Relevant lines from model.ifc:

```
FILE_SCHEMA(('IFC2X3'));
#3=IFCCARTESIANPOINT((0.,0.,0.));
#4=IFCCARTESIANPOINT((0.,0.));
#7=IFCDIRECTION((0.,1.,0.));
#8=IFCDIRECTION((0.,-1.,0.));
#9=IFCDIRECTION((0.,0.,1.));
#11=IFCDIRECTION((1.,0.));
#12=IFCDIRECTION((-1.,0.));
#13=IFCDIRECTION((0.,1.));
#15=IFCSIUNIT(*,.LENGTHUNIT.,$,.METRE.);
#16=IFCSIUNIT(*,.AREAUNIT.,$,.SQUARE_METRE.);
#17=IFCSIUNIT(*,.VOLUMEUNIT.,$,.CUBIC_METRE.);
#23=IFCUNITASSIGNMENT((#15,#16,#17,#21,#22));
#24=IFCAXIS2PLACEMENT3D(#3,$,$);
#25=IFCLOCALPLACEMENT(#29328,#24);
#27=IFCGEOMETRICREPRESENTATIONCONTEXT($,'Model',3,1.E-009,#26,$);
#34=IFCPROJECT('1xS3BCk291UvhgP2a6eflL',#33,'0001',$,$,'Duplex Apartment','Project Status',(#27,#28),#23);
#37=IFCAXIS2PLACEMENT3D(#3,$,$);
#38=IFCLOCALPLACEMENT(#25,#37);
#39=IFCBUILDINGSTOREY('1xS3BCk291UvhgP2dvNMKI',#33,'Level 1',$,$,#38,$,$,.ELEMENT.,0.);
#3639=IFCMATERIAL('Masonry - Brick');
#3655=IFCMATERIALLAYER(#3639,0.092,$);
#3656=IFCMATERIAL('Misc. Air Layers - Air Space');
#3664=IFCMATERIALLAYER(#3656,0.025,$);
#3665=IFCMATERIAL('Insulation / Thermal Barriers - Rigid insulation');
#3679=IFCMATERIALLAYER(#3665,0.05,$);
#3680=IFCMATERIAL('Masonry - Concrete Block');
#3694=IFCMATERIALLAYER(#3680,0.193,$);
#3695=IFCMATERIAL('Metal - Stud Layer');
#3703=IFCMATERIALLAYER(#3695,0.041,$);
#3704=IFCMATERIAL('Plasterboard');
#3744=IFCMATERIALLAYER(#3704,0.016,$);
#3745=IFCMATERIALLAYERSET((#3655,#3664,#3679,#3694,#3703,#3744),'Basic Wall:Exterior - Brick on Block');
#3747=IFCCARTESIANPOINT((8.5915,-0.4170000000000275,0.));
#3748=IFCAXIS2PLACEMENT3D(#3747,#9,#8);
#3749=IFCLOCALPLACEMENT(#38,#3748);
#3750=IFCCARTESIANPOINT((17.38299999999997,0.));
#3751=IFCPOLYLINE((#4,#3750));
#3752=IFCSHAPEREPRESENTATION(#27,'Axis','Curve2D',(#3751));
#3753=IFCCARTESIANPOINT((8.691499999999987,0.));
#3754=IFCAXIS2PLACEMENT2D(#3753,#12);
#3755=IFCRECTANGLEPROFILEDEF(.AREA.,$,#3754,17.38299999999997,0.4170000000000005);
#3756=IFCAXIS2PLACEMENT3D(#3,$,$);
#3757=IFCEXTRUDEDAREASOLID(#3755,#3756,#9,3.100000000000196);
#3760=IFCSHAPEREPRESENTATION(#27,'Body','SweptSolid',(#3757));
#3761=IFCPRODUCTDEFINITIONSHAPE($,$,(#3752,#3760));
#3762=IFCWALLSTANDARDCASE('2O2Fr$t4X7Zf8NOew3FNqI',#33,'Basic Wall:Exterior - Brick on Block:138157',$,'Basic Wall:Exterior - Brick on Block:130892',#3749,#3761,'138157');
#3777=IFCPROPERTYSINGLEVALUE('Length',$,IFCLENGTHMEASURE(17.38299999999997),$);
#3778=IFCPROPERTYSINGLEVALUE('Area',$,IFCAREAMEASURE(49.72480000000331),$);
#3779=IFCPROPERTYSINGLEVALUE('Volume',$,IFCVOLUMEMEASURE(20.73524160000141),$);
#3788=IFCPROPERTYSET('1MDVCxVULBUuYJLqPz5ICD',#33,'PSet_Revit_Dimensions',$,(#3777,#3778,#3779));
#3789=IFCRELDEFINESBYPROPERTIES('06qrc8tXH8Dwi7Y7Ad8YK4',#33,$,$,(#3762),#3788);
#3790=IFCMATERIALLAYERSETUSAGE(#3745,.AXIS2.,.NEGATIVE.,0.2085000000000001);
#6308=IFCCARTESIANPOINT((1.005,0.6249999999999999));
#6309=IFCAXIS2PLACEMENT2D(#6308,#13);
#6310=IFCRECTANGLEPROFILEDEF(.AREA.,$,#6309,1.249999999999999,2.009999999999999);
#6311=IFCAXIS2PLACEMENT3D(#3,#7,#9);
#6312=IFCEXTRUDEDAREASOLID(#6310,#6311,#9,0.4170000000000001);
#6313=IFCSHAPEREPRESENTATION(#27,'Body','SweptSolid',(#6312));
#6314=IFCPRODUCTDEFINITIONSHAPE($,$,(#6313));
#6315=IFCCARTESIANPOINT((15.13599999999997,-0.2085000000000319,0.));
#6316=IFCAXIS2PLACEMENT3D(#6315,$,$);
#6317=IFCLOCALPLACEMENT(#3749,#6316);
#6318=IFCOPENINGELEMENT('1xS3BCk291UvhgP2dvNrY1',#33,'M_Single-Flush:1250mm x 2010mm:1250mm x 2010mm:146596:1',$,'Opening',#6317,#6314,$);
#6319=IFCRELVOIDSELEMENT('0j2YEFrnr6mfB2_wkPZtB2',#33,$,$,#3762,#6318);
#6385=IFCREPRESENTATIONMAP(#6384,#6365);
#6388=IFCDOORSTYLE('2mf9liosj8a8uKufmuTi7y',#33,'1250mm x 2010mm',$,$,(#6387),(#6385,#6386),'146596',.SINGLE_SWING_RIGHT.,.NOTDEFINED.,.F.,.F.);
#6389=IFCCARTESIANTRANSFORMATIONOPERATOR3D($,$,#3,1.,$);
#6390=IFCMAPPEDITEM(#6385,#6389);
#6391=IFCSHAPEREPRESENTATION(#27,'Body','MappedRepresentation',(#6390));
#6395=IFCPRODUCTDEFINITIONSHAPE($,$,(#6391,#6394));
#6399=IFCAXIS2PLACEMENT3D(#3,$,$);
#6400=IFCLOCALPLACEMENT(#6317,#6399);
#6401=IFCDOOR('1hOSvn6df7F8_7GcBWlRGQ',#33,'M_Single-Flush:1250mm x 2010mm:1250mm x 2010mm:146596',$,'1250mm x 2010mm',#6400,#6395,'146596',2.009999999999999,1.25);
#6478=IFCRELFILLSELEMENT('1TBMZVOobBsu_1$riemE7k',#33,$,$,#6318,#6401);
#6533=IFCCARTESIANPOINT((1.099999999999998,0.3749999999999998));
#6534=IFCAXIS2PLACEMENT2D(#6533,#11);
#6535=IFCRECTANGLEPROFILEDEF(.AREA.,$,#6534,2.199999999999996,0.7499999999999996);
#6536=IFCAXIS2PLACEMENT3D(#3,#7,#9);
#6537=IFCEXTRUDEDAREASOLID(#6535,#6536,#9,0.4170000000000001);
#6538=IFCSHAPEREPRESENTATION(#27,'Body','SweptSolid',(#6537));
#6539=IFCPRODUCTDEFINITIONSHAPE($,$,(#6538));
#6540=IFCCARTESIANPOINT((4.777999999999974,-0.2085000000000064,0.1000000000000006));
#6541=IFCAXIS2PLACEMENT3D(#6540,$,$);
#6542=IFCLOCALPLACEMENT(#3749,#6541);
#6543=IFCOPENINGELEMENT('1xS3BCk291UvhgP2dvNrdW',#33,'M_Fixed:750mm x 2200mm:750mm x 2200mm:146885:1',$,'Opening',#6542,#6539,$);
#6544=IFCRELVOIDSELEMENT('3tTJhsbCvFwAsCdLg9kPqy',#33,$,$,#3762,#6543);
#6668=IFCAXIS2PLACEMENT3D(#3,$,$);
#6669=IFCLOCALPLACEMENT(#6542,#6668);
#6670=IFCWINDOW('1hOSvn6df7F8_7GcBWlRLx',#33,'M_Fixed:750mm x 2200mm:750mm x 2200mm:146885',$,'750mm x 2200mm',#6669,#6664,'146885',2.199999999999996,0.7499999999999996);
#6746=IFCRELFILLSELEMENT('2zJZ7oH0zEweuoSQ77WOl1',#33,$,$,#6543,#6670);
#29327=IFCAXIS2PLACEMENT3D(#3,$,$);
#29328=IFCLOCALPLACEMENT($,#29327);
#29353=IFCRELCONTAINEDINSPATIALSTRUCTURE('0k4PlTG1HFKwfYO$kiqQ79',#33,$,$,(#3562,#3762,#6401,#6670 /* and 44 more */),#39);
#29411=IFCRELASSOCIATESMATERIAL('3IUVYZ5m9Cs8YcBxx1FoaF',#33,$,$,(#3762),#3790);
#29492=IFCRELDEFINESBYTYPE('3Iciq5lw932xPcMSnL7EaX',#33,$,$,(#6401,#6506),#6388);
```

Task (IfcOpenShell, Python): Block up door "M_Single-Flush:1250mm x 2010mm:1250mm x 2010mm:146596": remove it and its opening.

```python
import ifcopenshell
import ifcopenshell.api.feature
import ifcopenshell.api.pset
import ifcopenshell.api.root
import ifcopenshell.geom
import ifcopenshell.util.element
import ifcopenshell.util.shape
import ifcopenshell.util.unit

model = ifcopenshell.open("model.ifc")
area_scale = ifcopenshell.util.unit.calculate_unit_scale(model, "AREAUNIT")
volume_scale = ifcopenshell.util.unit.calculate_unit_scale(model, "VOLUMEUNIT")
settings = ifcopenshell.geom.settings()


def volume(element):
    """Net volume in cubic metres, openings subtracted."""
    shape = ifcopenshell.geom.create_shape(settings, element)
    return ifcopenshell.util.shape.get_volume(shape.geometry)


door = model.by_guid("1hOSvn6df7F8_7GcBWlRGQ")
opening = door.FillsVoids[0].RelatingOpeningElement
wall = opening.VoidsElements[0].RelatingBuildingElement
before = volume(wall)

ifcopenshell.api.root.remove_product(model, product=door)
ifcopenshell.api.feature.remove_feature(model, feature=opening)

after = volume(wall)
thickness = 0.417  # wall thickness in metres

# Update the wall's stored quantities.
pset = model.by_id(ifcopenshell.util.element.get_pset(wall, "PSet_Revit_Dimensions", should_inherit=False)["id"])
ifcopenshell.api.pset.edit_pset(model, pset=pset, properties={
    "Area": model.create_entity("IfcAreaMeasure", after / thickness / area_scale),
    "Volume": model.create_entity("IfcVolumeMeasure", after / volume_scale),
})

print(f"wall volume {before:.3f} -> {after:.3f} m3")

model.write("model_rev.ifc")
```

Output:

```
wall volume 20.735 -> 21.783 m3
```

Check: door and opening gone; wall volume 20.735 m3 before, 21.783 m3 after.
